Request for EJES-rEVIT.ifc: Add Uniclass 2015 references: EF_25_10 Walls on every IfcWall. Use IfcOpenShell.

First a look at what the model holds.

```python
import ifcopenshell

model = ifcopenshell.open("EJES-rEVIT.ifc")
print(model.schema)
print("classifications:", [c.Name for c in model.by_type("IfcClassification")])
for ifc_class in ("IfcDoor", "IfcRoof", "IfcStair", "IfcWall", "IfcWindow"):
    print(ifc_class, len(model.by_type(ifc_class)))
```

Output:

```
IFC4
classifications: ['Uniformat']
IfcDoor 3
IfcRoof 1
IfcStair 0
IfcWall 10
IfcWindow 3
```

```python
import ifcopenshell
import ifcopenshell.api.classification

model = ifcopenshell.open("EJES-rEVIT.ifc")

system = ifcopenshell.api.classification.add_classification(model, classification="Uniclass 2015")

codes = {
    "IfcWall": ("EF_25_10", "Walls"),
}
for ifc_class, (code, name) in codes.items():
    products = model.by_type(ifc_class)
    ifcopenshell.api.classification.add_reference(
        model, products=products, classification=system, identification=code, name=name
    )
    print(code, len(products))

model.write("EJES-rEVIT_updated.ifc")
```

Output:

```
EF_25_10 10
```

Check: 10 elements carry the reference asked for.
